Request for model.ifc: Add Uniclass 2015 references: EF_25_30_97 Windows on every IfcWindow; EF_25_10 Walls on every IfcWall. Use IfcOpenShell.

First a look at what the model holds.

```python
import ifcopenshell

model = ifcopenshell.open("model.ifc")
print(model.schema)
print("classifications:", [c.Name for c in model.by_type("IfcClassification")])
for ifc_class in ("IfcDoor", "IfcRoof", "IfcStair", "IfcWall", "IfcWindow"):
    print(ifc_class, len(model.by_type(ifc_class)))
```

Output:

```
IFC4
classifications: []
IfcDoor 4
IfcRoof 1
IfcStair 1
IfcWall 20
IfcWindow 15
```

```python
import ifcopenshell
import ifcopenshell.api.classification

model = ifcopenshell.open("model.ifc")

system = ifcopenshell.api.classification.add_classification(model, classification="Uniclass 2015")

codes = {
    "IfcWindow": ("EF_25_30_97", "Windows"),
    "IfcWall": ("EF_25_10", "Walls"),
}
for ifc_class, (code, name) in codes.items():
    products = model.by_type(ifc_class)
    ifcopenshell.api.classification.add_reference(
        model, products=products, classification=system, identification=code, name=name
    )
    print(code, len(products))

model.write("model_edited.ifc")
```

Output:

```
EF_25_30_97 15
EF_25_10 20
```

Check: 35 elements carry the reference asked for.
